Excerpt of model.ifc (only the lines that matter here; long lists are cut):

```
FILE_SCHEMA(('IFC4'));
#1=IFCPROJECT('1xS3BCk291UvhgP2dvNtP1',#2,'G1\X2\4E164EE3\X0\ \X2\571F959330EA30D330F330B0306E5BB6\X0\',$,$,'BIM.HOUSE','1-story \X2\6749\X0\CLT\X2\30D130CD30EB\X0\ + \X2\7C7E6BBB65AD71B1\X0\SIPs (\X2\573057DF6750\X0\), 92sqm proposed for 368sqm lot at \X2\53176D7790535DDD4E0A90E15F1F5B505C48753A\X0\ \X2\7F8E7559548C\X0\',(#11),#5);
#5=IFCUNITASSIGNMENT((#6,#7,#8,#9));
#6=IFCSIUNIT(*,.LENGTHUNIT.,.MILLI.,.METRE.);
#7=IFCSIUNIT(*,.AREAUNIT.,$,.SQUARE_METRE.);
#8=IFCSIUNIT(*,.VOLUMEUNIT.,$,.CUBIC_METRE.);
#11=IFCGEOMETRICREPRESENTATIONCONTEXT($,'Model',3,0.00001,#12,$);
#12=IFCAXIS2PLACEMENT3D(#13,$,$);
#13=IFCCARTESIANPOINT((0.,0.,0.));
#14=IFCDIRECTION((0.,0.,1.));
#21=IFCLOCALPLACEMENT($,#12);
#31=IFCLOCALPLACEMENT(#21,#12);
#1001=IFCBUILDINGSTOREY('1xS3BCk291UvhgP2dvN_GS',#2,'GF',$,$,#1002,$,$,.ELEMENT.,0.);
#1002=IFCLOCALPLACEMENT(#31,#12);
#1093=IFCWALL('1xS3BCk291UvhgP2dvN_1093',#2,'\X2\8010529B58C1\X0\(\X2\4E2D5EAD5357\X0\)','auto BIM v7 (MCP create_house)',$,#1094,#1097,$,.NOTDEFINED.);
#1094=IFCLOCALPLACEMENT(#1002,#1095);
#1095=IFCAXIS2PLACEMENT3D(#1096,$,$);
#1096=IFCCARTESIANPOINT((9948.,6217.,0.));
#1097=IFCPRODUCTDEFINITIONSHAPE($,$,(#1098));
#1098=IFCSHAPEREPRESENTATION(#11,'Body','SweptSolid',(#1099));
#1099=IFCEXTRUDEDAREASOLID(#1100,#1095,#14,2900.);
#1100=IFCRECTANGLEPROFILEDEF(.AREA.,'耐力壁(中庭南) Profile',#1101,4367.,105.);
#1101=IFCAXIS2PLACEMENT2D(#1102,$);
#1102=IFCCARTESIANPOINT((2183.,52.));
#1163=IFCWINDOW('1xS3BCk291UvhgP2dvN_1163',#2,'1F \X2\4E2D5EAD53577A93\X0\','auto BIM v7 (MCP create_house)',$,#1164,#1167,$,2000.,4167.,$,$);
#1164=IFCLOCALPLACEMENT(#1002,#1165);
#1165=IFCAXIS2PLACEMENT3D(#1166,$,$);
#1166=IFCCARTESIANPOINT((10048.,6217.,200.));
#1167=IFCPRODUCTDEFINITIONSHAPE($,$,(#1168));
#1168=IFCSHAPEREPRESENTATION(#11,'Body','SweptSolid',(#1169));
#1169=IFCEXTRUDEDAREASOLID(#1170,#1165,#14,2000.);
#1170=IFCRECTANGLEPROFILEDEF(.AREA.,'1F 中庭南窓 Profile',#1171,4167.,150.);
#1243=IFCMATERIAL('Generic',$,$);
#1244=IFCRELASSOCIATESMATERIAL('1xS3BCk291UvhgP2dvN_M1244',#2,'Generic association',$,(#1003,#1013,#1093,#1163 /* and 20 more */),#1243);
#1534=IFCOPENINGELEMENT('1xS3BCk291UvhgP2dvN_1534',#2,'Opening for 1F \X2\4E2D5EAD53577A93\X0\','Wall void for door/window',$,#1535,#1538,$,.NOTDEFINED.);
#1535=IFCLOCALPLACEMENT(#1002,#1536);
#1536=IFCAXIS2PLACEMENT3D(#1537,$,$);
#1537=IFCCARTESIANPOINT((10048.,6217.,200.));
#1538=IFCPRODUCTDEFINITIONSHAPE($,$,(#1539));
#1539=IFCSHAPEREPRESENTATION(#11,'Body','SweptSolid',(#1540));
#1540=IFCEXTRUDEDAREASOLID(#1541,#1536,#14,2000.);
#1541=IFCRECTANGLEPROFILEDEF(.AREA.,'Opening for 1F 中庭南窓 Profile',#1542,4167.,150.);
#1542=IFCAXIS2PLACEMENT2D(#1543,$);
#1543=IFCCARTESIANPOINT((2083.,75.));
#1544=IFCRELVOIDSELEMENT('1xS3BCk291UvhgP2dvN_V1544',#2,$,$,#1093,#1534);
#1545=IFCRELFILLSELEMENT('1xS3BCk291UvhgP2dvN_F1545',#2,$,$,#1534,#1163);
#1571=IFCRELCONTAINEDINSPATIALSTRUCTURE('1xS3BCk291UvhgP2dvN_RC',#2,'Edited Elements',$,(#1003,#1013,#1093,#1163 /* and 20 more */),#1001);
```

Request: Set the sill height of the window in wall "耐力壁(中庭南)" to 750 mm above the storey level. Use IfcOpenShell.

```python
import numpy as np
import ifcopenshell
import ifcopenshell.api.geometry
import ifcopenshell.geom
import ifcopenshell.util.element
import ifcopenshell.util.placement
import ifcopenshell.util.shape
import ifcopenshell.util.unit

model = ifcopenshell.open("model.ifc")
unit_scale = ifcopenshell.util.unit.calculate_unit_scale(model)

window = model.by_guid("1xS3BCk291UvhgP2dvN_1163")
opening = window.FillsVoids[0].RelatingOpeningElement
storey = ifcopenshell.util.element.get_container(window, ifc_class="IfcBuildingStorey")
level = ifcopenshell.util.placement.get_local_placement(storey.ObjectPlacement)[2, 3]

# The opening's origin need not be at the sill, so measure its lowest point.
shape = ifcopenshell.geom.create_shape(ifcopenshell.geom.settings(), opening)
bottom = ifcopenshell.util.shape.get_shape_bottom_elevation(shape, shape.geometry) / unit_scale
dz = level + 750.0 - bottom

shift = np.array([0.0, 0.0, dz])
# The window is not placed relative to its opening, so move both.
for product in (opening, window):
    matrix = ifcopenshell.util.placement.get_local_placement(product.ObjectPlacement)
    matrix[:3, 3] += shift
    ifcopenshell.api.geometry.edit_object_placement(model, product=product, matrix=matrix, is_si=False)

print(f"moved by {dz * unit_scale:+.3f} m")

model.write("model_edited.ifc")
```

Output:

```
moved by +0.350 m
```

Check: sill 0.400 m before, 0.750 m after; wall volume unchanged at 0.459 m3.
